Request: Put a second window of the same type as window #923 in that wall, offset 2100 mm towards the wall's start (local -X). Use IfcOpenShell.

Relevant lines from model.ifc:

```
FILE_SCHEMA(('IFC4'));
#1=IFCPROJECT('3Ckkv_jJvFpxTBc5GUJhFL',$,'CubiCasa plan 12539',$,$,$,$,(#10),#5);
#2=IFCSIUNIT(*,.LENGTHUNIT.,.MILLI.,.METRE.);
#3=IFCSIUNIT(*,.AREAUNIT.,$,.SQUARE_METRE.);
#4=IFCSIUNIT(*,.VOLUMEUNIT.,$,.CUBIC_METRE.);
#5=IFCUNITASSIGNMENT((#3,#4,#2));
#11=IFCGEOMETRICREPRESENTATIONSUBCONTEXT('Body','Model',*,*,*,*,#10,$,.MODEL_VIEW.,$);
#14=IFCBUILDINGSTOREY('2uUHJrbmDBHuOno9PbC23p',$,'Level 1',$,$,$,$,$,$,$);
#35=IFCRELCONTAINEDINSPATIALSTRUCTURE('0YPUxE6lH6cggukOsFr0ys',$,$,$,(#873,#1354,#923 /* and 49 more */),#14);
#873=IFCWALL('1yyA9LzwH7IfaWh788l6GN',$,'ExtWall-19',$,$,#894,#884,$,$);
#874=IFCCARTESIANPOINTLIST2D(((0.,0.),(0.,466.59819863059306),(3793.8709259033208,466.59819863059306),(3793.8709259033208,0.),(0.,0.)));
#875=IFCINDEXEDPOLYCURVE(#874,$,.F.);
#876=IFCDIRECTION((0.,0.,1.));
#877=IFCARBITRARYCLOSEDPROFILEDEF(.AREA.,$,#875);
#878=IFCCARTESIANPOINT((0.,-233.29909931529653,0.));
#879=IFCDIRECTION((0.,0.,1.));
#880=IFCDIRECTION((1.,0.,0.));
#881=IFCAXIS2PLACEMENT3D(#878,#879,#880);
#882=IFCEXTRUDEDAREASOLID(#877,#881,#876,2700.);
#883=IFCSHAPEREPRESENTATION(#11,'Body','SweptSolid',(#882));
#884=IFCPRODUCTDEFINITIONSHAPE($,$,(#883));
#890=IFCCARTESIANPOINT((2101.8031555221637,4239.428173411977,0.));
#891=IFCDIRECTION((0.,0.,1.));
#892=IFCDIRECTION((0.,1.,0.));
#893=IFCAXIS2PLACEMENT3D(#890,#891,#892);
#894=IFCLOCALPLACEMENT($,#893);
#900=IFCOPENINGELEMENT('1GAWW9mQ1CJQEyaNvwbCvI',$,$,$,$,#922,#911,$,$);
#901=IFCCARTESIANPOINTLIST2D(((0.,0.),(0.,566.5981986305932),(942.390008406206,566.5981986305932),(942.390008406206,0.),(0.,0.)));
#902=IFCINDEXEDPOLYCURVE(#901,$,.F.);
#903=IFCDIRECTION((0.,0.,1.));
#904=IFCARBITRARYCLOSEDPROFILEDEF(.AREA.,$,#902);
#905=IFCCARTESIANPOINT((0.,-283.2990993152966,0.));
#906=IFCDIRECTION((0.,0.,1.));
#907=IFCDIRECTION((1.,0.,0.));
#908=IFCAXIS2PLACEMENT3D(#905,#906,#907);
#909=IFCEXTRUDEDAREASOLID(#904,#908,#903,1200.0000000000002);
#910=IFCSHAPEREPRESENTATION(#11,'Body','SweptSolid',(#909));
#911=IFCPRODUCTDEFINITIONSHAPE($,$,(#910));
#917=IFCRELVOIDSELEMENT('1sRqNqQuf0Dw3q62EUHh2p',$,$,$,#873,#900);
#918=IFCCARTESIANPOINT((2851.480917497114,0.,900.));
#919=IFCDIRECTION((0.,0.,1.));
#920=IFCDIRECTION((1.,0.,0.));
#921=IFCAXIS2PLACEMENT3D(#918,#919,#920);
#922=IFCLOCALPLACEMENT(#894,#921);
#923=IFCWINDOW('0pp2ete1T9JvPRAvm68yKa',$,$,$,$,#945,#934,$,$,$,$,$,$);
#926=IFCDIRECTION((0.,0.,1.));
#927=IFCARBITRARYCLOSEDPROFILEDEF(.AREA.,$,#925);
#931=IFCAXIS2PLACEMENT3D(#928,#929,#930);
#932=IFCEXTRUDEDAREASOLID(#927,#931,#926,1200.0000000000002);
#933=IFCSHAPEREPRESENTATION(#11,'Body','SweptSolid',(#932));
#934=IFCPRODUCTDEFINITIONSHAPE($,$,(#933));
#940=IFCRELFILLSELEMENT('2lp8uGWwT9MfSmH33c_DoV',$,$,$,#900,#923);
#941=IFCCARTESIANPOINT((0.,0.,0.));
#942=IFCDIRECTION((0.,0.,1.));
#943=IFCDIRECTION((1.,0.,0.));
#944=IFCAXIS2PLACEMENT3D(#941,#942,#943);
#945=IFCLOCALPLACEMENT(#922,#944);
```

```python
import ifcopenshell
import ifcopenshell.api.feature
import ifcopenshell.api.geometry
import ifcopenshell.api.root
import ifcopenshell.geom
import ifcopenshell.util.element
import ifcopenshell.util.placement
import ifcopenshell.util.shape
import ifcopenshell.util.unit

model = ifcopenshell.open("model.ifc")
unit_scale = ifcopenshell.util.unit.calculate_unit_scale(model)
settings = ifcopenshell.geom.settings()


def volume(element):
    """Net volume in cubic metres, openings subtracted."""
    shape = ifcopenshell.geom.create_shape(settings, element)
    return ifcopenshell.util.shape.get_volume(shape.geometry)


window = model.by_id(923)
opening = window.FillsVoids[0].RelatingOpeningElement
wall = opening.VoidsElements[0].RelatingBuildingElement
before = volume(wall)
shift = ifcopenshell.util.placement.get_local_placement(wall.ObjectPlacement)[:3, 0] * -2.1 / unit_scale

# copy_class copies the void relationship, type, container and properties, but no geometry.
new_opening = ifcopenshell.api.root.copy_class(model, product=opening)
new_opening.Representation = ifcopenshell.util.element.copy_deep(
    model, opening.Representation, exclude=["IfcGeometricRepresentationContext", "IfcRepresentationMap"]
)
new_window = ifcopenshell.api.root.copy_class(model, product=window)
new_window.Representation = ifcopenshell.util.element.copy_deep(
    model, window.Representation, exclude=["IfcGeometricRepresentationContext", "IfcRepresentationMap"]
)
ifcopenshell.api.feature.add_filling(model, opening=new_opening, element=new_window)

for old, new in ((opening, new_opening), (window, new_window)):
    matrix = ifcopenshell.util.placement.get_local_placement(old.ObjectPlacement)
    matrix[:3, 3] += shift
    ifcopenshell.api.geometry.edit_object_placement(model, product=new, matrix=matrix, is_si=False)

after = volume(wall)

print(f"wall volume {before:.3f} -> {after:.3f} m3")

model.write("model_rev.ifc")
```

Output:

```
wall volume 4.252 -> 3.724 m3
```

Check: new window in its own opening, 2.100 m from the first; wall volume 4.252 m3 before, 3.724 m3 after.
